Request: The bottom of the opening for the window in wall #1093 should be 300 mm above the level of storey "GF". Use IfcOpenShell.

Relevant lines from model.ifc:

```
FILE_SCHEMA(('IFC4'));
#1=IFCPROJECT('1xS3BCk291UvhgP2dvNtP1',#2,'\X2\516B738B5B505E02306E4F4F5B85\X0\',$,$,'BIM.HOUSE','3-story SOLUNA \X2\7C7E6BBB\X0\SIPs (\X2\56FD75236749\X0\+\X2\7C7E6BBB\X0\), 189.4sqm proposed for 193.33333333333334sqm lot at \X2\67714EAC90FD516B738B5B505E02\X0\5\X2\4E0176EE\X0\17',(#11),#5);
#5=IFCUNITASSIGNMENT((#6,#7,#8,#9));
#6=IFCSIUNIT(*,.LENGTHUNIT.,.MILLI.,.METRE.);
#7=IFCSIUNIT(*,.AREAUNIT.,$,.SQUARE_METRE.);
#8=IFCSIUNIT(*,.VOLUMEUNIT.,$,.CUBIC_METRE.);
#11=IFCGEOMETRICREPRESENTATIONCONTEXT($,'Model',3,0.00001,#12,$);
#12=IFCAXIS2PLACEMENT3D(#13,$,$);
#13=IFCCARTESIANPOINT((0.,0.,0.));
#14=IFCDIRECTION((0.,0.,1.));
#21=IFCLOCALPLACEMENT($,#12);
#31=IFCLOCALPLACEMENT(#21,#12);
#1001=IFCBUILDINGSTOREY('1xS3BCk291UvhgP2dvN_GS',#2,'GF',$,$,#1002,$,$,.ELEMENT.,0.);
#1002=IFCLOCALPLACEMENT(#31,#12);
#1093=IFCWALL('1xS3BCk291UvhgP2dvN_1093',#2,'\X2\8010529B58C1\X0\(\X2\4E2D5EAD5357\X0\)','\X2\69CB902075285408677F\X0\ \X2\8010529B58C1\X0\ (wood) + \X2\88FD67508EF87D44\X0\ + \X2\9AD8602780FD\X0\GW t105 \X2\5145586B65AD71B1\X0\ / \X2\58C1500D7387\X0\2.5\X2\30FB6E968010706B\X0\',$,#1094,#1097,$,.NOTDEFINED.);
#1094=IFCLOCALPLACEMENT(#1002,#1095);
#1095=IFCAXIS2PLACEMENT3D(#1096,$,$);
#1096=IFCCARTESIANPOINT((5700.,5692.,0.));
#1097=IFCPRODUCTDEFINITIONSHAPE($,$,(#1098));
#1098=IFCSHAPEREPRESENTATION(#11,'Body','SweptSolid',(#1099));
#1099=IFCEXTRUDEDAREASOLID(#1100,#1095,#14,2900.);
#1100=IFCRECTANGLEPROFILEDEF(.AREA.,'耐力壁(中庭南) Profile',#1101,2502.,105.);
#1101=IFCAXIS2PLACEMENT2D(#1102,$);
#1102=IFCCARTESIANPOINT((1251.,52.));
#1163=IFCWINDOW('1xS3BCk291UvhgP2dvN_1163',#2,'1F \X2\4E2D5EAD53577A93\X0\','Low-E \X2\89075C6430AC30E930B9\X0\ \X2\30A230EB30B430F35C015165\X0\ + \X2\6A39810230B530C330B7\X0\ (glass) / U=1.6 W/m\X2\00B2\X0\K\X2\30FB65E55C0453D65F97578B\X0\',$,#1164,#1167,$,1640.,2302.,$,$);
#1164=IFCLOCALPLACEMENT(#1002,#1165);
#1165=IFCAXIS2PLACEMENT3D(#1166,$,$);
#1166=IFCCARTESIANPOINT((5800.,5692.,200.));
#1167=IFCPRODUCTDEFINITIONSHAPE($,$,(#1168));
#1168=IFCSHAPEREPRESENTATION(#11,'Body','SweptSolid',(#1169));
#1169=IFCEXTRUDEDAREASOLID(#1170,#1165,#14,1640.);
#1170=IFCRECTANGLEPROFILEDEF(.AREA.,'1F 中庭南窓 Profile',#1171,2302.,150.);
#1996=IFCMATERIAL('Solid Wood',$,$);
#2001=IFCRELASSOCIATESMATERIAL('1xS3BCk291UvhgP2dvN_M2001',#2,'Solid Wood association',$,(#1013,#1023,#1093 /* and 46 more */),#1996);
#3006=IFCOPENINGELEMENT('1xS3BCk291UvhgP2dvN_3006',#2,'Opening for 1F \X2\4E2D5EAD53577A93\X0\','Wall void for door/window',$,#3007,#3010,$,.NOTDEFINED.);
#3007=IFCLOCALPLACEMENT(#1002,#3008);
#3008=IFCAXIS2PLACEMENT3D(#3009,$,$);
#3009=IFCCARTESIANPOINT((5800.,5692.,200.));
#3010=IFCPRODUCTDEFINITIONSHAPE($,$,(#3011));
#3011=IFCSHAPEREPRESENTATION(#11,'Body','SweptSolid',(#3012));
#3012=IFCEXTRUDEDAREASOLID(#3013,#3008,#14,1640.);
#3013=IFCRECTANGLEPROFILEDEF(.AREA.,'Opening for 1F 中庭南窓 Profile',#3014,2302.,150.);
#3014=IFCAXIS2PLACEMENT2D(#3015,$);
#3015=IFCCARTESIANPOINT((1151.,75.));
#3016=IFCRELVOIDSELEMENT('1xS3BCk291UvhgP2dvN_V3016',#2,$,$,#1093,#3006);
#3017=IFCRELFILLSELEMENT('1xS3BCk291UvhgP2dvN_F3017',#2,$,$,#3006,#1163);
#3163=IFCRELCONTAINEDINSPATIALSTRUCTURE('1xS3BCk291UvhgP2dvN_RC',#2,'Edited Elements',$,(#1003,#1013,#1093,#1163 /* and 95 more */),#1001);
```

```python
import numpy as np
import ifcopenshell
import ifcopenshell.api.geometry
import ifcopenshell.geom
import ifcopenshell.util.element
import ifcopenshell.util.placement
import ifcopenshell.util.shape
import ifcopenshell.util.unit

model = ifcopenshell.open("model.ifc")
unit_scale = ifcopenshell.util.unit.calculate_unit_scale(model)

window = model.by_guid("1xS3BCk291UvhgP2dvN_1163")
opening = window.FillsVoids[0].RelatingOpeningElement
storey = ifcopenshell.util.element.get_container(window, ifc_class="IfcBuildingStorey")
level = ifcopenshell.util.placement.get_local_placement(storey.ObjectPlacement)[2, 3]

# The opening's origin need not be at the sill, so measure its lowest point.
shape = ifcopenshell.geom.create_shape(ifcopenshell.geom.settings(), opening)
bottom = ifcopenshell.util.shape.get_shape_bottom_elevation(shape, shape.geometry) / unit_scale
dz = level + 300.0 - bottom

shift = np.array([0.0, 0.0, dz])
# The window is not placed relative to its opening, so move both.
for product in (opening, window):
    matrix = ifcopenshell.util.placement.get_local_placement(product.ObjectPlacement)
    matrix[:3, 3] += shift
    ifcopenshell.api.geometry.edit_object_placement(model, product=product, matrix=matrix, is_si=False)

print(f"moved by {dz * unit_scale:+.3f} m")

model.write("model_rev.ifc")
```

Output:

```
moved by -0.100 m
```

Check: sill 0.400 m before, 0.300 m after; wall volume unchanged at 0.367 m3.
